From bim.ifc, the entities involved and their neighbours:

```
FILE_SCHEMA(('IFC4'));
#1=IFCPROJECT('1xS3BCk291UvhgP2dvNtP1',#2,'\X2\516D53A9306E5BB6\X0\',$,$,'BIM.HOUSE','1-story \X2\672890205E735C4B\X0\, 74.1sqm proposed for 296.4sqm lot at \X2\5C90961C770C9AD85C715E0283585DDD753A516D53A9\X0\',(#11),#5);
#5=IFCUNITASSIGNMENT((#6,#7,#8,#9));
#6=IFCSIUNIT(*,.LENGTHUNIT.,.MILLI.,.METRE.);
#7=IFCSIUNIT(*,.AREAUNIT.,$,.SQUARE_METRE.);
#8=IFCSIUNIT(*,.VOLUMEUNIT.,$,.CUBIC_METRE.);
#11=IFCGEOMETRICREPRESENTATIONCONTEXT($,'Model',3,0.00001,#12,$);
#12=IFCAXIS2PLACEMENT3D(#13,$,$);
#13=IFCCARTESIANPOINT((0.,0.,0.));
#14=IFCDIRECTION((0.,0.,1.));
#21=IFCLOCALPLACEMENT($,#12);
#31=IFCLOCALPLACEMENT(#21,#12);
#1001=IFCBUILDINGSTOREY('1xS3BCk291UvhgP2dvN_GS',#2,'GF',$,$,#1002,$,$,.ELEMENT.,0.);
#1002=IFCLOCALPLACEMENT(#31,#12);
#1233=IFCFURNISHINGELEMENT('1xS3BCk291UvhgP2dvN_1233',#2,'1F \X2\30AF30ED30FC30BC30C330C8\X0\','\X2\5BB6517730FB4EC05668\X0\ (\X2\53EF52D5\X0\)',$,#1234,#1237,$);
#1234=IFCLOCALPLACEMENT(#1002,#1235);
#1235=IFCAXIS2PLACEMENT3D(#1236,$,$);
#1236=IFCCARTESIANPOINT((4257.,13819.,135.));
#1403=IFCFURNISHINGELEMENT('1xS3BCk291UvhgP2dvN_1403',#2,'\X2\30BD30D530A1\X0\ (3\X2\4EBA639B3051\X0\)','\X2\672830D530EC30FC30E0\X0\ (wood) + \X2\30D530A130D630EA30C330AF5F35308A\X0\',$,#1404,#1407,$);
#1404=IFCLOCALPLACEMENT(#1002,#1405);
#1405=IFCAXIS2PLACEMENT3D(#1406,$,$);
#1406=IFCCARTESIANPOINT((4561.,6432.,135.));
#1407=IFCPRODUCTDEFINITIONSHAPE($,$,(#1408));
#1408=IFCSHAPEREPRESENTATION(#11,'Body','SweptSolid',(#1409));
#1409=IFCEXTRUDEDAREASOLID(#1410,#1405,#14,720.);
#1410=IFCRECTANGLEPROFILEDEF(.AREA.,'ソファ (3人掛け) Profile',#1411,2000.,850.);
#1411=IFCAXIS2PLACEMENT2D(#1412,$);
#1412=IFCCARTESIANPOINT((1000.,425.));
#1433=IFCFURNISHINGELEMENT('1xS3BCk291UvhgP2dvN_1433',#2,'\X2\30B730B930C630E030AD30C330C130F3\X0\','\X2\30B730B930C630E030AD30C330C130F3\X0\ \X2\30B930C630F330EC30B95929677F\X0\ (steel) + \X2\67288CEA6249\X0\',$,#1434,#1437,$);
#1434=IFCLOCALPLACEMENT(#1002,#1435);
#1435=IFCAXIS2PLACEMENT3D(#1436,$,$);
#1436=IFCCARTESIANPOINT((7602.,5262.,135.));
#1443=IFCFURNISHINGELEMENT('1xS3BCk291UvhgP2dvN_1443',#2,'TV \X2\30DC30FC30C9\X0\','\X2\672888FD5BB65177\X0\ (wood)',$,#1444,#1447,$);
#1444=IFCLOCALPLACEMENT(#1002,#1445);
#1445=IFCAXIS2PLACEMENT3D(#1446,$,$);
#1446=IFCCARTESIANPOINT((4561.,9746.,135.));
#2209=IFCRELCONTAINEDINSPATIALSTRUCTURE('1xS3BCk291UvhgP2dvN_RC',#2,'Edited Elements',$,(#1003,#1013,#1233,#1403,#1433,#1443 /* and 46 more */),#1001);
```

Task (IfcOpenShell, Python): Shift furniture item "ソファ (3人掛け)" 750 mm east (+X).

```python
import ifcopenshell
import ifcopenshell.api.geometry
import ifcopenshell.util.placement
import ifcopenshell.util.unit

model = ifcopenshell.open("bim.ifc")
unit_scale = ifcopenshell.util.unit.calculate_unit_scale(model)

item = model.by_guid("1xS3BCk291UvhgP2dvN_1403")
matrix = ifcopenshell.util.placement.get_local_placement(item.ObjectPlacement)
matrix[0, 3] += 0.75 / unit_scale
ifcopenshell.api.geometry.edit_object_placement(model, product=item, matrix=matrix, is_si=False)

print(ifcopenshell.util.placement.get_local_placement(item.ObjectPlacement).round(3) + 0.0)

model.write("bim_edited.ifc")
```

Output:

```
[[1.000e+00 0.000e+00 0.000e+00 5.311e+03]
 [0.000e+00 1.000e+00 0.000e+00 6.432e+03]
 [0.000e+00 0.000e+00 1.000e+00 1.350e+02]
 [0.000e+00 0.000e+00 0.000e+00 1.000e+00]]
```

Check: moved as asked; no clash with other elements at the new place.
